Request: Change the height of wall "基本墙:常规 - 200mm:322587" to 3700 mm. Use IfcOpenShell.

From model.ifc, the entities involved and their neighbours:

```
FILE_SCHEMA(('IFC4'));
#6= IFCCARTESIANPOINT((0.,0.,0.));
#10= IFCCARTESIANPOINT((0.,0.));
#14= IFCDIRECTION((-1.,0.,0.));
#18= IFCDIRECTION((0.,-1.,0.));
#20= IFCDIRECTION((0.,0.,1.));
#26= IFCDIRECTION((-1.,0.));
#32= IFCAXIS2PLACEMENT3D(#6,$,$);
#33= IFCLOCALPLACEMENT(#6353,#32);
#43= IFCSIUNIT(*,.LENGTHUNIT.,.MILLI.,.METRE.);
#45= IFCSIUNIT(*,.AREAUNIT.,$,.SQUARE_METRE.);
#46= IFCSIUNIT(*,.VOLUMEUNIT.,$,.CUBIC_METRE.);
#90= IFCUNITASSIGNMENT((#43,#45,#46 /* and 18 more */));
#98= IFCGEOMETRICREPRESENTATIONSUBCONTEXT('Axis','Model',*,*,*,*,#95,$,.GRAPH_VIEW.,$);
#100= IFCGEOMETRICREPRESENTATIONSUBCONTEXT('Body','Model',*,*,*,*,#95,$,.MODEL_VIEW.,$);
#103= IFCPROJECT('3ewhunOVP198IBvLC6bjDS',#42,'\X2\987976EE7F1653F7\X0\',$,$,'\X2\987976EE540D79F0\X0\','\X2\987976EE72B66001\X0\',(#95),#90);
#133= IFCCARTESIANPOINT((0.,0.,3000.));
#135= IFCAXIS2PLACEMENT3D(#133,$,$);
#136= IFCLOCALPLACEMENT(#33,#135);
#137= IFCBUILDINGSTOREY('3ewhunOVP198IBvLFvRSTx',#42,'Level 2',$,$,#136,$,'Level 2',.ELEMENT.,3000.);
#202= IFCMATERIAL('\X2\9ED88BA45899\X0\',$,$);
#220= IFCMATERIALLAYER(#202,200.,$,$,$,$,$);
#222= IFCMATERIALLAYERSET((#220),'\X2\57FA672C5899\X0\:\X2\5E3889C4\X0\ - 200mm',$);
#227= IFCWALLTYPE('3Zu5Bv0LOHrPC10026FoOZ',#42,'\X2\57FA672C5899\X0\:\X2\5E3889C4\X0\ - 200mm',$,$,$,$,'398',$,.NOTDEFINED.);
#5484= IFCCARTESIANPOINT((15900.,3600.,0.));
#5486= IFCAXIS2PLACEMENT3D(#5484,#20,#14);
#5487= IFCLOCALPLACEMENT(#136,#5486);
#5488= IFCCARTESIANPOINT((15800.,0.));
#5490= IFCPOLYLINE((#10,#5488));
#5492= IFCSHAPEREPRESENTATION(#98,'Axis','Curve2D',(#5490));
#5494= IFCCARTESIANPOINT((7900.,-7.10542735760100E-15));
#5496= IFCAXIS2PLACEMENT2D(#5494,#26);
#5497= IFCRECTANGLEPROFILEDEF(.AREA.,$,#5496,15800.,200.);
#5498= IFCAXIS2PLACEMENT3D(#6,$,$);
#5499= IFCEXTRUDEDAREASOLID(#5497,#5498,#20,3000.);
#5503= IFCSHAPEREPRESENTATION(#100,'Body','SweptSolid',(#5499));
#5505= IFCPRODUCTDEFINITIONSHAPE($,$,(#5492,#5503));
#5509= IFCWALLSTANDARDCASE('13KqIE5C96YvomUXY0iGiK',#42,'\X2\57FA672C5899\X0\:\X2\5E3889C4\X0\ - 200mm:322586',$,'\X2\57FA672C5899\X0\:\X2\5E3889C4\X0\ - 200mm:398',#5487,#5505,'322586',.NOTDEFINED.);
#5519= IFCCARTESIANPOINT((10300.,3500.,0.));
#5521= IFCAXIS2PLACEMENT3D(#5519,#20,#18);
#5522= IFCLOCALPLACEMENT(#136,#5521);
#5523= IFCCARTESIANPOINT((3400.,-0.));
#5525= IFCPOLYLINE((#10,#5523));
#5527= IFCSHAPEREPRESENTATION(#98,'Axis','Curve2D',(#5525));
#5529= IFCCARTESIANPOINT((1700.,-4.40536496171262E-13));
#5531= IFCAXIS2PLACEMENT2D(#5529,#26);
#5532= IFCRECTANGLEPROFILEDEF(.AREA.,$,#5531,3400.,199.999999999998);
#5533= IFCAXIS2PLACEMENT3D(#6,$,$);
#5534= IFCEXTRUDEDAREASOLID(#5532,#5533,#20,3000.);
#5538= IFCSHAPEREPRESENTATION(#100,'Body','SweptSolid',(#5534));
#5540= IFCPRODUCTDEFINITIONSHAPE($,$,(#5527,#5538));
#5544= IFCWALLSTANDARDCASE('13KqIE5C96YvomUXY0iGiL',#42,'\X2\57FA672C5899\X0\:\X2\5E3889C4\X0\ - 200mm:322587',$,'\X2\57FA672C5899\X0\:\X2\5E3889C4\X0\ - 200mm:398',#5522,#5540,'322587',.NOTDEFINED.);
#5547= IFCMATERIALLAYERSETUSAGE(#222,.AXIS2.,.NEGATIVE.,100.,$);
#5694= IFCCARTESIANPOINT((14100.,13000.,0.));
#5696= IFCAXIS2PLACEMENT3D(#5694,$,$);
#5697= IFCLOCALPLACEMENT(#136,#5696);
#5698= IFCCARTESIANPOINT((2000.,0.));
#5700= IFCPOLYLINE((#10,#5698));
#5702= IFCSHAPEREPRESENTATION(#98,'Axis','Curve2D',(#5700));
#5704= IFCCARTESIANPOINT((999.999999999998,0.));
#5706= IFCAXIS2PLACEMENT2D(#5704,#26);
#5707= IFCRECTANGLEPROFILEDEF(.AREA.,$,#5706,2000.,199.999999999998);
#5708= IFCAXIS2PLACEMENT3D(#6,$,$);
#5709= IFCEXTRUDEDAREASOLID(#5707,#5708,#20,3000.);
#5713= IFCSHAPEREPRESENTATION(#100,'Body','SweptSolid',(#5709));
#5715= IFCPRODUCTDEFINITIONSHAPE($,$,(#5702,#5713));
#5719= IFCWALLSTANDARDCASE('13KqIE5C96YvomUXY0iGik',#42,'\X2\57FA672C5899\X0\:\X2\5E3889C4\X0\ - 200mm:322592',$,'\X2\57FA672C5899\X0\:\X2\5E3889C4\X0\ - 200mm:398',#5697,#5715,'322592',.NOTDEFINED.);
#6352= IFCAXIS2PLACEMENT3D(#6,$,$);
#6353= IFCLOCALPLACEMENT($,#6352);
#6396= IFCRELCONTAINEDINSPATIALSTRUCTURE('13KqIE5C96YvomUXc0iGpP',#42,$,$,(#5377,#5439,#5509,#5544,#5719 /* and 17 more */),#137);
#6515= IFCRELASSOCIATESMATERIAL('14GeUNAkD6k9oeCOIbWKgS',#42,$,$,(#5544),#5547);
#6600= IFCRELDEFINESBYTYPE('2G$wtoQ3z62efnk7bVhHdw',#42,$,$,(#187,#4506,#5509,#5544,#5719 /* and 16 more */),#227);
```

```python
import ifcopenshell
import ifcopenshell.geom
import ifcopenshell.util.representation
import ifcopenshell.util.shape

model = ifcopenshell.open("model.ifc")
settings = ifcopenshell.geom.settings()


def volume(element):
    """Net volume in cubic metres, openings subtracted."""
    shape = ifcopenshell.geom.create_shape(settings, element)
    return ifcopenshell.util.shape.get_volume(shape.geometry)


wall = model.by_guid("13KqIE5C96YvomUXY0iGiL")
before = volume(wall)

body = ifcopenshell.util.representation.get_representation(wall, "Model", "Body")
solid = body.Items[0]
old_height = solid.Depth
solid.Depth = 3700.0
after = volume(wall)

print(f"height {old_height:g} -> {solid.Depth:g}, volume {before:.3f} -> {after:.3f} m3")

model.write("model_updated.ifc")
```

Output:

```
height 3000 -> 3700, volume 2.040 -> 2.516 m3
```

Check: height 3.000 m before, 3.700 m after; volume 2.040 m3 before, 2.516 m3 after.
